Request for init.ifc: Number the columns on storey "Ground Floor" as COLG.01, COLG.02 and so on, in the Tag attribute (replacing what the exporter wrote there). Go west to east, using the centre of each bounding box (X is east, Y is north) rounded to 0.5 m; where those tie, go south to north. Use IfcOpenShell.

First a look at what the model holds.

```python
import ifcopenshell
import ifcopenshell.util.element
import ifcopenshell.util.placement

model = ifcopenshell.open("init.ifc")
print(model.schema)
storey = next(s for s in model.by_type("IfcBuildingStorey") if s.Name == "Ground Floor")
columns = [e for e in ifcopenshell.util.element.get_decomposition(storey) if e.is_a("IfcColumn")]
for e in sorted(columns, key=lambda e: e.id()):
    origin = ifcopenshell.util.placement.get_local_placement(e.ObjectPlacement)[:3, 3]
    print(e.id(), e.Tag, e.Name, origin.round(2) + 0.0, sep=" | ")
```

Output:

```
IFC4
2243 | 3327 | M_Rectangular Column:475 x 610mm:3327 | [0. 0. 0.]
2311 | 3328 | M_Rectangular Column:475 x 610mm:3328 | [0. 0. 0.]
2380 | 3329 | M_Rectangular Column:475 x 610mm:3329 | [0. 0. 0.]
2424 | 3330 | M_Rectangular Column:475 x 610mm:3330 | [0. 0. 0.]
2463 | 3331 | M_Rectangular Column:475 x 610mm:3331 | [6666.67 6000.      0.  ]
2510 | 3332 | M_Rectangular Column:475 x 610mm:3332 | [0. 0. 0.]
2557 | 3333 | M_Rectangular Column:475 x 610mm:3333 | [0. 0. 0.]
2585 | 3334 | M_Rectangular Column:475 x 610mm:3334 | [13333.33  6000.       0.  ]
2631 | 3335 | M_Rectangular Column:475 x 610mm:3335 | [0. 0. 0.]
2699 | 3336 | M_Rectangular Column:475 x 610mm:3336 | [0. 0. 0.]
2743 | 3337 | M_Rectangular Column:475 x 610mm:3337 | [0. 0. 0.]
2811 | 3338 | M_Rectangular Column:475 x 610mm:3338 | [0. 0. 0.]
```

```python
import ifcopenshell
import ifcopenshell.geom
import ifcopenshell.util.element
import ifcopenshell.util.shape

model = ifcopenshell.open("init.ifc")
settings = ifcopenshell.geom.settings()
settings.set("use-world-coords", True)


def centre(element):
    shape = ifcopenshell.geom.create_shape(settings, element)
    return ifcopenshell.util.shape.get_bbox_centroid(shape.geometry)


storey = next(s for s in model.by_type("IfcBuildingStorey") if s.Name == "Ground Floor")
columns = [e for e in ifcopenshell.util.element.get_decomposition(storey) if e.is_a("IfcColumn")]

# Insertion points can sit at a corner or the storey origin, so sort by the geometry (in metres).
centres = {e: centre(e) for e in columns}
columns.sort(key=lambda e: (round(centres[e][0] / 0.5), centres[e][1]))

for i, e in enumerate(columns, start=1):
    number = f"COLG.{i:02d}"
    e.Tag = number
    print(e.id(), number)

model.write("init_updated.ifc")
```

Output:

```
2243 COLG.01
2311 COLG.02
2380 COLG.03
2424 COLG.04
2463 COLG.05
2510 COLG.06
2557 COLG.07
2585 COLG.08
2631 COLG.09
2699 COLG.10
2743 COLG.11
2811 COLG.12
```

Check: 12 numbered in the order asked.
